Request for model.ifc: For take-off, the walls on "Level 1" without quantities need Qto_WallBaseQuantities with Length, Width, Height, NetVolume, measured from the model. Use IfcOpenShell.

First a look at what the model holds.

```python
import ifcopenshell
import ifcopenshell.util.element
import ifcopenshell.util.unit

model = ifcopenshell.open("model.ifc")
print(model.schema)
for unit_type in ("LENGTHUNIT", "AREAUNIT", "VOLUMEUNIT"):
    print(unit_type, ifcopenshell.util.unit.calculate_unit_scale(model, unit_type))
storey = next(s for s in model.by_type("IfcBuildingStorey") if s.Name == "Level 1")
walls = [e for e in ifcopenshell.util.element.get_decomposition(storey) if e.is_a("IfcWall")]
for e in sorted(walls, key=lambda e: e.id()):
    print(e.id(), e.is_a(), e.Name, list(ifcopenshell.util.element.get_psets(e, qtos_only=True)), sep=" | ")
```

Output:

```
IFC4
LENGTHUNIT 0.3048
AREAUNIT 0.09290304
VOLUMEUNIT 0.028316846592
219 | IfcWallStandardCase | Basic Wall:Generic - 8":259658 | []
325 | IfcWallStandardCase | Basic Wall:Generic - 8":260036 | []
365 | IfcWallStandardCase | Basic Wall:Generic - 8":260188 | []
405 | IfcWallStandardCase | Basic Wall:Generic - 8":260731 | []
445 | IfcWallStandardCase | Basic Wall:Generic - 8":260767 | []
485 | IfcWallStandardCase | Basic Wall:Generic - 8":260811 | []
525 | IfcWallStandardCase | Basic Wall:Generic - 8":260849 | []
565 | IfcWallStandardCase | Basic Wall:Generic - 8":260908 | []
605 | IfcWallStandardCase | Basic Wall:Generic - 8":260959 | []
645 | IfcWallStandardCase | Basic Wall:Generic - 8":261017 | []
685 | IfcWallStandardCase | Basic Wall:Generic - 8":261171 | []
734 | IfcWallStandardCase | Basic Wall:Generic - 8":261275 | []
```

```python
import ifcopenshell
import ifcopenshell.api.pset
import ifcopenshell.geom
import ifcopenshell.util.element
import ifcopenshell.util.shape
import ifcopenshell.util.unit

model = ifcopenshell.open("model.ifc")
unit_scale = ifcopenshell.util.unit.calculate_unit_scale(model)
volume_scale = ifcopenshell.util.unit.calculate_unit_scale(model, "VOLUMEUNIT")
settings = ifcopenshell.geom.settings()

storey = next(s for s in model.by_type("IfcBuildingStorey") if s.Name == "Level 1")
walls = [e for e in ifcopenshell.util.element.get_decomposition(storey) if e.is_a("IfcWall")]

for e in sorted(walls, key=lambda e: e.id()):
    if ifcopenshell.util.element.get_psets(e, qtos_only=True, should_inherit=False):
        continue
    # Geometry comes back in metres, in the element's own axes.
    shape = ifcopenshell.geom.create_shape(settings, e)
    values = {
        "Length": ifcopenshell.util.shape.get_x(shape.geometry) / unit_scale,
        "Width": ifcopenshell.util.shape.get_y(shape.geometry) / unit_scale,
        "Height": ifcopenshell.util.shape.get_z(shape.geometry) / unit_scale,
        "NetVolume": ifcopenshell.util.shape.get_volume(shape.geometry) / volume_scale,
    }
    qto = ifcopenshell.api.pset.add_qto(model, product=e, name="Qto_WallBaseQuantities")
    ifcopenshell.api.pset.edit_qto(model, qto=qto, properties=values)
    print(e.id(), {k: round(v, 3) for k, v in values.items()})

model.write("model_updated.ifc")
```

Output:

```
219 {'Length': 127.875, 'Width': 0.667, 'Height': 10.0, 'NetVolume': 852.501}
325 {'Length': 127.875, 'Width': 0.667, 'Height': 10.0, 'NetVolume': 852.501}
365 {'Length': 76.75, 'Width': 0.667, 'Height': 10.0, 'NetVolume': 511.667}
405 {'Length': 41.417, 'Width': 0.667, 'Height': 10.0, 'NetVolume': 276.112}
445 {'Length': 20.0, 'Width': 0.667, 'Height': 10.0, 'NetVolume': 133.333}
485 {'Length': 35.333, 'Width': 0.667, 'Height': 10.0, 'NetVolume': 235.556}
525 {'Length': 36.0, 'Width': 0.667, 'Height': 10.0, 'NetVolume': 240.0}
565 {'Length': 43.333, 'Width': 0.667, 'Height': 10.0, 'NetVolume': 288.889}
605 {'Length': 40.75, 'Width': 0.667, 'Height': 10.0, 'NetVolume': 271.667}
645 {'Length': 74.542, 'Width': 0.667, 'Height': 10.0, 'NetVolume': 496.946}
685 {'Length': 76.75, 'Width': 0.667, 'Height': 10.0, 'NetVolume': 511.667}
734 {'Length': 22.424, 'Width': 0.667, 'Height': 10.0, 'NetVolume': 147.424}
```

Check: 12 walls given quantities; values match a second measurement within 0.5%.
